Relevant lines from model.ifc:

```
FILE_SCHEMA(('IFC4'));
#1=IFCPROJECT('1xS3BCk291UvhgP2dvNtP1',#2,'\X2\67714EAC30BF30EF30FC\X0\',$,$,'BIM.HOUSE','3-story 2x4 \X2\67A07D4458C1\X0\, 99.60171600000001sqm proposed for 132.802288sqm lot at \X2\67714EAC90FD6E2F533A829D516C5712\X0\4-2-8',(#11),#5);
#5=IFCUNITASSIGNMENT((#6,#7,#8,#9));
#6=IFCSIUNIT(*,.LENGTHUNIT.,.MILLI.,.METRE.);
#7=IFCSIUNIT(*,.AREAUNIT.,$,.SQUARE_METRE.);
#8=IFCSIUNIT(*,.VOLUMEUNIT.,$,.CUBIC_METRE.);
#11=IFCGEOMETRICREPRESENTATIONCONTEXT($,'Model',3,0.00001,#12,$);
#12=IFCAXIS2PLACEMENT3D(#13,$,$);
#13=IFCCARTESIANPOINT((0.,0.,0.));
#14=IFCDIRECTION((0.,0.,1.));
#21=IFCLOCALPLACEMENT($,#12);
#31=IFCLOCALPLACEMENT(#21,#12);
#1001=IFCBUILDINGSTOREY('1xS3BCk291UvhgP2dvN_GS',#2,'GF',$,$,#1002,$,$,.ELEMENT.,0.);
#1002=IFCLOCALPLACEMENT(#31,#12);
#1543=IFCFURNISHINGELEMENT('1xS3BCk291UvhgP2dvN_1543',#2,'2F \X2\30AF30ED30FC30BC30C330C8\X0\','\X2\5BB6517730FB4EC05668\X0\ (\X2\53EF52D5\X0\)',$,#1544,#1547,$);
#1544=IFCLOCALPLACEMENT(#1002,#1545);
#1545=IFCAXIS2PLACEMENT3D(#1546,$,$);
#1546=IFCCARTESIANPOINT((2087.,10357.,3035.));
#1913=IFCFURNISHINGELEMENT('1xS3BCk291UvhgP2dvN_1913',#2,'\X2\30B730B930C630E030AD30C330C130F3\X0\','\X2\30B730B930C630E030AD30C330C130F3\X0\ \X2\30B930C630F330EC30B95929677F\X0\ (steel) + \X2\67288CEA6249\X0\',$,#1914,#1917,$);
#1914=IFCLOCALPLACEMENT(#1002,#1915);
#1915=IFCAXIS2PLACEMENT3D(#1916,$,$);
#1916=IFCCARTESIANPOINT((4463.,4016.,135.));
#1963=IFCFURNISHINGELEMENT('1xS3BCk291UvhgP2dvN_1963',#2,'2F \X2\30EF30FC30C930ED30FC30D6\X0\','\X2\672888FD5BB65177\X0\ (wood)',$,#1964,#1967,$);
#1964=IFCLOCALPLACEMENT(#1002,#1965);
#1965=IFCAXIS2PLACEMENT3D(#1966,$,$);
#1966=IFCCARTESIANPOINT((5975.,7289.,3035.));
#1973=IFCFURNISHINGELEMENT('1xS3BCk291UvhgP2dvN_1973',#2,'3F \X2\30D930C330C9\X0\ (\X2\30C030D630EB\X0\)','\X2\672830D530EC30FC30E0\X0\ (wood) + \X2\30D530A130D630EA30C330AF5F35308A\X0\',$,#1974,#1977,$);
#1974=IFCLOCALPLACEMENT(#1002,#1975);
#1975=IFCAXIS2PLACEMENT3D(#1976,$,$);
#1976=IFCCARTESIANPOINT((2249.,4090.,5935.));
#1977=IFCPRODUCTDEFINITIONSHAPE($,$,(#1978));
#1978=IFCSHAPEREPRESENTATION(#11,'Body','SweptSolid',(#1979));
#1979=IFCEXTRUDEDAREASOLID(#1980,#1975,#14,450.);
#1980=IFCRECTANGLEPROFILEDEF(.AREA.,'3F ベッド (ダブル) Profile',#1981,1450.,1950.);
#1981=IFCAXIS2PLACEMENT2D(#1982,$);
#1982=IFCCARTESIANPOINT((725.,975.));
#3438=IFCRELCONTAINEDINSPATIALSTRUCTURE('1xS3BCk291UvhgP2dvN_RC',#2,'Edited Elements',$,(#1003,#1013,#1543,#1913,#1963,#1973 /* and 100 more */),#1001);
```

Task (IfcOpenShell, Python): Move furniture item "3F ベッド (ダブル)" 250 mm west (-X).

```python
import ifcopenshell
import ifcopenshell.api.geometry
import ifcopenshell.util.placement

model = ifcopenshell.open("model.ifc")

item = model.by_id(1973)
matrix = ifcopenshell.util.placement.get_local_placement(item.ObjectPlacement)
matrix[0, 3] -= 250.0
ifcopenshell.api.geometry.edit_object_placement(model, product=item, matrix=matrix, is_si=False)

print(ifcopenshell.util.placement.get_local_placement(item.ObjectPlacement).round(3) + 0.0)

model.write("model_rev.ifc")
```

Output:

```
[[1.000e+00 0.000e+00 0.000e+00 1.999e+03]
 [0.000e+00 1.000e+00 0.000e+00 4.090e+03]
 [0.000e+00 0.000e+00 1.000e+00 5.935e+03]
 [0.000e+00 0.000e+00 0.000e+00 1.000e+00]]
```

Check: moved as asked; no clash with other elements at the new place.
